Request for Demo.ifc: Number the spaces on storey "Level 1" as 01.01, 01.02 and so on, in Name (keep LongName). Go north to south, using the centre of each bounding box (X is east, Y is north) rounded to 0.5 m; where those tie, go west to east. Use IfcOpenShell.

First a look at what the model holds.

```python
import ifcopenshell
import ifcopenshell.util.element
import ifcopenshell.util.placement

model = ifcopenshell.open("Demo.ifc")
print(model.schema)
storey = next(s for s in model.by_type("IfcBuildingStorey") if s.Name == "Level 1")
spaces = [e for e in ifcopenshell.util.element.get_decomposition(storey) if e.is_a("IfcSpace")]
for e in sorted(spaces, key=lambda e: e.id()):
    origin = ifcopenshell.util.placement.get_local_placement(e.ObjectPlacement)[:3, 3]
    print(e.id(), e.Name, e.LongName, origin.round(2) + 0.0, sep=" | ")
```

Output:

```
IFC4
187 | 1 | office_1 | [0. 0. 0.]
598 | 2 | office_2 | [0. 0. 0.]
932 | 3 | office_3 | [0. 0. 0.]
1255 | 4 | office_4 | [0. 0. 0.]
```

```python
import ifcopenshell
import ifcopenshell.geom
import ifcopenshell.util.element
import ifcopenshell.util.shape

model = ifcopenshell.open("Demo.ifc")
settings = ifcopenshell.geom.settings()
settings.set("use-world-coords", True)


def centre(element):
    shape = ifcopenshell.geom.create_shape(settings, element)
    return ifcopenshell.util.shape.get_bbox_centroid(shape.geometry)


storey = next(s for s in model.by_type("IfcBuildingStorey") if s.Name == "Level 1")
spaces = [e for e in ifcopenshell.util.element.get_decomposition(storey) if e.is_a("IfcSpace")]

# Insertion points can sit at a corner or the storey origin, so sort by the geometry (in metres).
centres = {e: centre(e) for e in spaces}
spaces.sort(key=lambda e: (-round(centres[e][1] / 0.5), centres[e][0]))

for i, e in enumerate(spaces, start=1):
    number = f"01.{i:02d}"
    e.Name = number
    print(e.id(), number)

model.write("Demo-out.ifc")
```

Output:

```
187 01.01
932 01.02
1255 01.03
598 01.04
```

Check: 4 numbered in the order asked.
